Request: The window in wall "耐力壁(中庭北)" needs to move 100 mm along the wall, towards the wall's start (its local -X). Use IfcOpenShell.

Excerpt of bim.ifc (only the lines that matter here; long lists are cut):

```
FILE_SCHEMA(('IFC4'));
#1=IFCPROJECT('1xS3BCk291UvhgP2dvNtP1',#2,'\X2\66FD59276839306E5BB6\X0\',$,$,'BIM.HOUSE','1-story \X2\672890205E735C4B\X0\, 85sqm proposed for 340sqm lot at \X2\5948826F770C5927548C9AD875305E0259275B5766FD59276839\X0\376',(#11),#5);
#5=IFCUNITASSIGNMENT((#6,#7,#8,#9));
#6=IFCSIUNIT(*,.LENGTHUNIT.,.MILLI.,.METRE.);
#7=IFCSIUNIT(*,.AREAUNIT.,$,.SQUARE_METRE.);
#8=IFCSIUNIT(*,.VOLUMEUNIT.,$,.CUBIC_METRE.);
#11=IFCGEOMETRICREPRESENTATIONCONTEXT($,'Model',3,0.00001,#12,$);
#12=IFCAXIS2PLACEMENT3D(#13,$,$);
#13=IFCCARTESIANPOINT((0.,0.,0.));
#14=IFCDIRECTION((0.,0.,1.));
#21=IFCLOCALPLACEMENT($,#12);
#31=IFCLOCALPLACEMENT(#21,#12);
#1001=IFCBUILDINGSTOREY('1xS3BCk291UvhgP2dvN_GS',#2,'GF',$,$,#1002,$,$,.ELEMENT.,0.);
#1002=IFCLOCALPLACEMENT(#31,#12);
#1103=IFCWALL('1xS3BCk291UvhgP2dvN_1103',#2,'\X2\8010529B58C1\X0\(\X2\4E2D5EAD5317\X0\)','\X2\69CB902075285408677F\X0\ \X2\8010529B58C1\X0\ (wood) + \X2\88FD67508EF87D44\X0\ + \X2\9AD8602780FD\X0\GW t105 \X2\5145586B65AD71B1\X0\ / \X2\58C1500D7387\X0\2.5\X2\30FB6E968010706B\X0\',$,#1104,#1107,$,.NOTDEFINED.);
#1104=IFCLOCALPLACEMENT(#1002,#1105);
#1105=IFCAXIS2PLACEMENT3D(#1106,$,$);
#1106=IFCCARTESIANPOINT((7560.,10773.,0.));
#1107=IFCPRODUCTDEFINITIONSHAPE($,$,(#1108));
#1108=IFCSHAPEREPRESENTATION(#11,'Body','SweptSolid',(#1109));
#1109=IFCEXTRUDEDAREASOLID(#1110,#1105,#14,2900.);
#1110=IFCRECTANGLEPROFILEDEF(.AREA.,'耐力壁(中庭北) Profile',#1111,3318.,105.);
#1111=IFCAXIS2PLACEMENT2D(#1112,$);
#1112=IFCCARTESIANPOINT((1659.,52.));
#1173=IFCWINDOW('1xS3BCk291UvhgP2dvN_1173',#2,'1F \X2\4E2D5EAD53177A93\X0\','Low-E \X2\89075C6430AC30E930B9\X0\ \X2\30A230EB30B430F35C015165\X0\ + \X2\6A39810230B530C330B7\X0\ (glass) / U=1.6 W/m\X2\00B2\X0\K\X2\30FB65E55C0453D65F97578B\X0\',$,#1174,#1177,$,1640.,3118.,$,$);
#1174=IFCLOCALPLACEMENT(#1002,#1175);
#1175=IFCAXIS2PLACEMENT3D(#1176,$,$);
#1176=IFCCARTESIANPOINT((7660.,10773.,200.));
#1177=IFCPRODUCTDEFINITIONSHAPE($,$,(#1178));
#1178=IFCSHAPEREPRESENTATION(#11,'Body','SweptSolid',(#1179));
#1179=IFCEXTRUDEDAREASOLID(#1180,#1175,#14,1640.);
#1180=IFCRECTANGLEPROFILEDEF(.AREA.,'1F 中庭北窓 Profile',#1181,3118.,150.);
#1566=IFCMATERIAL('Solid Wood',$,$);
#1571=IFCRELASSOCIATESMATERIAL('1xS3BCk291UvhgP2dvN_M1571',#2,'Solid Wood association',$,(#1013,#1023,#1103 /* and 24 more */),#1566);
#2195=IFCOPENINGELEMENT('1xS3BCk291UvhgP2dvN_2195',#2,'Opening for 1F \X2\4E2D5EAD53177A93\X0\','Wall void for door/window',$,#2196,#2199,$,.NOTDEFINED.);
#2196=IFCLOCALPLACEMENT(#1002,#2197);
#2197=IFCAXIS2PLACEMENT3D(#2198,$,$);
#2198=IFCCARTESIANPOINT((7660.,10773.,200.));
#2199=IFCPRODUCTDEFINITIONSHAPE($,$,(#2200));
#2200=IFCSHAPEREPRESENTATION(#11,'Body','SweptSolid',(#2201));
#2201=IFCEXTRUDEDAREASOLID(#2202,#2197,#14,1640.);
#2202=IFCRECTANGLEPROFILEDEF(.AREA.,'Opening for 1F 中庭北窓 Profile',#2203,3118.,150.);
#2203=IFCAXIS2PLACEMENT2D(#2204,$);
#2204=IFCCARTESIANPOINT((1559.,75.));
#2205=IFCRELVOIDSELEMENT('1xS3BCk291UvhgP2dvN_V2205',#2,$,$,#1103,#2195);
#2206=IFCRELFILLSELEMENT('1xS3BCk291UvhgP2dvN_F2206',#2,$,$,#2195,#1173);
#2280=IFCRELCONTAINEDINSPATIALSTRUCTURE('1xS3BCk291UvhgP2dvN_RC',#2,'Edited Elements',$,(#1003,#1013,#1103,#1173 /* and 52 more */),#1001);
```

```python
import ifcopenshell
import ifcopenshell.api.geometry
import ifcopenshell.util.placement
import ifcopenshell.util.unit

model = ifcopenshell.open("bim.ifc")
unit_scale = ifcopenshell.util.unit.calculate_unit_scale(model)

window = model.by_guid("1xS3BCk291UvhgP2dvN_1173")
opening = window.FillsVoids[0].RelatingOpeningElement
wall = opening.VoidsElements[0].RelatingBuildingElement

wall_matrix = ifcopenshell.util.placement.get_local_placement(wall.ObjectPlacement)
shift = wall_matrix[:3, 0] * -0.1 / unit_scale
before = ifcopenshell.util.placement.get_local_placement(window.ObjectPlacement)[:3, 3].copy()

# The window is not placed relative to its opening, so move both.
for product in (opening, window):
    matrix = ifcopenshell.util.placement.get_local_placement(product.ObjectPlacement)
    matrix[:3, 3] += shift
    ifcopenshell.api.geometry.edit_object_placement(model, product=product, matrix=matrix, is_si=False)

after = ifcopenshell.util.placement.get_local_placement(window.ObjectPlacement)[:3, 3]
print("window moved by", (after - before).round(3) + 0.0)

model.write("bim_updated.ifc")
```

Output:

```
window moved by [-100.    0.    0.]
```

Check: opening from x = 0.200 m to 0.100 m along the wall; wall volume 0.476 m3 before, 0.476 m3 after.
